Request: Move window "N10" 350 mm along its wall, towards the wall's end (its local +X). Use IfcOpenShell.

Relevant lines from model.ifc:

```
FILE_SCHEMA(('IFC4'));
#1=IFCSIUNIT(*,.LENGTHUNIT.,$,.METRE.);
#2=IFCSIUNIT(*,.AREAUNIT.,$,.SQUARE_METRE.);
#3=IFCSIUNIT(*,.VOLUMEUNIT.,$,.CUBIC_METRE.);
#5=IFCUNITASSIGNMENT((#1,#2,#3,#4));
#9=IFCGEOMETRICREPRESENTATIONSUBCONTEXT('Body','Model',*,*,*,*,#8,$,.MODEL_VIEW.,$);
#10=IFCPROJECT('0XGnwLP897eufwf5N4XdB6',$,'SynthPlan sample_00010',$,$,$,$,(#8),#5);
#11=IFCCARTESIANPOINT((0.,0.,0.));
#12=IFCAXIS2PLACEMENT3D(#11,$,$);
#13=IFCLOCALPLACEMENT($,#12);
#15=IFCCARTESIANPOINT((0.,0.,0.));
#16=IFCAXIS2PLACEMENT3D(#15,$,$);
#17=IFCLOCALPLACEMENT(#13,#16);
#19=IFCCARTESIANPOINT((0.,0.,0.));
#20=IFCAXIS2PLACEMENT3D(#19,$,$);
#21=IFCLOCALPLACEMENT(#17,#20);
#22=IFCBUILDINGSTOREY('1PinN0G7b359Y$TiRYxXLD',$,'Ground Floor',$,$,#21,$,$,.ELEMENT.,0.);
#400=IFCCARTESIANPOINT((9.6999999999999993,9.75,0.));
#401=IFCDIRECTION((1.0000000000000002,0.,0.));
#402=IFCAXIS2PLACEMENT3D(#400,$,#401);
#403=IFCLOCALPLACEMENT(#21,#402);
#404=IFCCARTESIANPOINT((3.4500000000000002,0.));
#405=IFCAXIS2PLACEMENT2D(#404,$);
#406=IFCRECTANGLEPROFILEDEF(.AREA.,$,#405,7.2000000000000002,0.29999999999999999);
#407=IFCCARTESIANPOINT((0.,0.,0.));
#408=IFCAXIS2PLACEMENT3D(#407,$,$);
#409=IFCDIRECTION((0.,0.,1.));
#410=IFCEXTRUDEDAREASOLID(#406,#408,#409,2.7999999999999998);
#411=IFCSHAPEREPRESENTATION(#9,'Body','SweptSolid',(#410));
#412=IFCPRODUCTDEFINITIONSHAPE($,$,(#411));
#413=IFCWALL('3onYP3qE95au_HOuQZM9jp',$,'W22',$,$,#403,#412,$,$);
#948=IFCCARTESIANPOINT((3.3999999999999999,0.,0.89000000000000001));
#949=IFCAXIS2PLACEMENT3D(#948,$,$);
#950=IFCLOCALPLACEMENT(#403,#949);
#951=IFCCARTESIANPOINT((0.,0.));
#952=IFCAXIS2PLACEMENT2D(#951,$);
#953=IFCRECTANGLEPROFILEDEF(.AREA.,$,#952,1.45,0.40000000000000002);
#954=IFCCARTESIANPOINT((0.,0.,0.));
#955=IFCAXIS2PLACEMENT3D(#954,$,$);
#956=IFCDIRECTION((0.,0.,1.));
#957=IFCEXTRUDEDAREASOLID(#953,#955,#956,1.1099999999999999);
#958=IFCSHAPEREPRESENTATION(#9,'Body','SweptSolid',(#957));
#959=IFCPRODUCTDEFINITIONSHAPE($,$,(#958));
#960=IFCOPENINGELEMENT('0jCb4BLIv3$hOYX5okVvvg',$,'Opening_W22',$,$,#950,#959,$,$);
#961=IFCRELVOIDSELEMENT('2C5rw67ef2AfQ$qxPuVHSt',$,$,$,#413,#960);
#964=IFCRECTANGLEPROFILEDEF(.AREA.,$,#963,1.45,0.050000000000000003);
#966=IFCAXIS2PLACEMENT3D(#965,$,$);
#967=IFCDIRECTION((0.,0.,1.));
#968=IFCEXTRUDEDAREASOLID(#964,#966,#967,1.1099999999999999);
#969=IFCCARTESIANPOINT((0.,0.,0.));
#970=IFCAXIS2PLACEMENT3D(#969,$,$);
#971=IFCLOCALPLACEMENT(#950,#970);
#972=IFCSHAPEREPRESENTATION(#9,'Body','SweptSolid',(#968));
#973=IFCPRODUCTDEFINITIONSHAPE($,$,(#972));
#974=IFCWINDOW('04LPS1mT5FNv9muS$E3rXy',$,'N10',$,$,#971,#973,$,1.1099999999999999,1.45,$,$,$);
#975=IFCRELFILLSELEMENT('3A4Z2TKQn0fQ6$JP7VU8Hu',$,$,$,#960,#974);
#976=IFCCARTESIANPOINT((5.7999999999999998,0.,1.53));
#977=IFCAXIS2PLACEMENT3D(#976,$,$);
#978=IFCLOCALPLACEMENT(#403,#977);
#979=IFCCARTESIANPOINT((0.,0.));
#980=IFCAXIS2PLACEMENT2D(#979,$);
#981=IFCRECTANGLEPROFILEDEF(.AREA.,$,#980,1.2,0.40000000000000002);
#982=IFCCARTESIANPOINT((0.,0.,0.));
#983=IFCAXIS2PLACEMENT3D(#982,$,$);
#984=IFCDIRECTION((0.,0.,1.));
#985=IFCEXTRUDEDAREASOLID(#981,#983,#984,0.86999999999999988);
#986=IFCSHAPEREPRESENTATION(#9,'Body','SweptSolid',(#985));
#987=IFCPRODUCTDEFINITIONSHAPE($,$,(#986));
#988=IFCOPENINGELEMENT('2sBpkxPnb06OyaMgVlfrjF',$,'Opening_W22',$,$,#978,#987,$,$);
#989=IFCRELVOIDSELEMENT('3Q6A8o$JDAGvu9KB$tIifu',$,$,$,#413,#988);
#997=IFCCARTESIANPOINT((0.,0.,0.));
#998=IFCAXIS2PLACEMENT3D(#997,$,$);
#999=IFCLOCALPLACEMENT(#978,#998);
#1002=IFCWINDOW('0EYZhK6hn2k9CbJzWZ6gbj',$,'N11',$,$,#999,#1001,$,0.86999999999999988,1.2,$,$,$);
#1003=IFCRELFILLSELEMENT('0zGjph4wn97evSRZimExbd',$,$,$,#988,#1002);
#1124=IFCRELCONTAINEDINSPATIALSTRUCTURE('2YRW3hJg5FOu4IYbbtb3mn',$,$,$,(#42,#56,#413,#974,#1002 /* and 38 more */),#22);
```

```python
import ifcopenshell
import ifcopenshell.api.geometry
import ifcopenshell.util.placement
import ifcopenshell.util.unit

model = ifcopenshell.open("model.ifc")
unit_scale = ifcopenshell.util.unit.calculate_unit_scale(model)

window = model.by_guid("04LPS1mT5FNv9muS$E3rXy")
opening = window.FillsVoids[0].RelatingOpeningElement
wall = opening.VoidsElements[0].RelatingBuildingElement

wall_matrix = ifcopenshell.util.placement.get_local_placement(wall.ObjectPlacement)
shift = wall_matrix[:3, 0] * 0.35 / unit_scale
before = ifcopenshell.util.placement.get_local_placement(window.ObjectPlacement)[:3, 3].copy()

# The window is placed relative to its opening, so it follows when the opening moves.
matrix = ifcopenshell.util.placement.get_local_placement(opening.ObjectPlacement)
matrix[:3, 3] += shift
ifcopenshell.api.geometry.edit_object_placement(
    model, product=opening, matrix=matrix, is_si=False, should_transform_children=True
)

after = ifcopenshell.util.placement.get_local_placement(window.ObjectPlacement)[:3, 3]
print("window moved by", (after - before).round(3) + 0.0)

model.write("model-out.ifc")
```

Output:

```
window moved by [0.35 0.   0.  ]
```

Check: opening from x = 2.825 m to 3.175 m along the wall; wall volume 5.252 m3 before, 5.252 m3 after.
